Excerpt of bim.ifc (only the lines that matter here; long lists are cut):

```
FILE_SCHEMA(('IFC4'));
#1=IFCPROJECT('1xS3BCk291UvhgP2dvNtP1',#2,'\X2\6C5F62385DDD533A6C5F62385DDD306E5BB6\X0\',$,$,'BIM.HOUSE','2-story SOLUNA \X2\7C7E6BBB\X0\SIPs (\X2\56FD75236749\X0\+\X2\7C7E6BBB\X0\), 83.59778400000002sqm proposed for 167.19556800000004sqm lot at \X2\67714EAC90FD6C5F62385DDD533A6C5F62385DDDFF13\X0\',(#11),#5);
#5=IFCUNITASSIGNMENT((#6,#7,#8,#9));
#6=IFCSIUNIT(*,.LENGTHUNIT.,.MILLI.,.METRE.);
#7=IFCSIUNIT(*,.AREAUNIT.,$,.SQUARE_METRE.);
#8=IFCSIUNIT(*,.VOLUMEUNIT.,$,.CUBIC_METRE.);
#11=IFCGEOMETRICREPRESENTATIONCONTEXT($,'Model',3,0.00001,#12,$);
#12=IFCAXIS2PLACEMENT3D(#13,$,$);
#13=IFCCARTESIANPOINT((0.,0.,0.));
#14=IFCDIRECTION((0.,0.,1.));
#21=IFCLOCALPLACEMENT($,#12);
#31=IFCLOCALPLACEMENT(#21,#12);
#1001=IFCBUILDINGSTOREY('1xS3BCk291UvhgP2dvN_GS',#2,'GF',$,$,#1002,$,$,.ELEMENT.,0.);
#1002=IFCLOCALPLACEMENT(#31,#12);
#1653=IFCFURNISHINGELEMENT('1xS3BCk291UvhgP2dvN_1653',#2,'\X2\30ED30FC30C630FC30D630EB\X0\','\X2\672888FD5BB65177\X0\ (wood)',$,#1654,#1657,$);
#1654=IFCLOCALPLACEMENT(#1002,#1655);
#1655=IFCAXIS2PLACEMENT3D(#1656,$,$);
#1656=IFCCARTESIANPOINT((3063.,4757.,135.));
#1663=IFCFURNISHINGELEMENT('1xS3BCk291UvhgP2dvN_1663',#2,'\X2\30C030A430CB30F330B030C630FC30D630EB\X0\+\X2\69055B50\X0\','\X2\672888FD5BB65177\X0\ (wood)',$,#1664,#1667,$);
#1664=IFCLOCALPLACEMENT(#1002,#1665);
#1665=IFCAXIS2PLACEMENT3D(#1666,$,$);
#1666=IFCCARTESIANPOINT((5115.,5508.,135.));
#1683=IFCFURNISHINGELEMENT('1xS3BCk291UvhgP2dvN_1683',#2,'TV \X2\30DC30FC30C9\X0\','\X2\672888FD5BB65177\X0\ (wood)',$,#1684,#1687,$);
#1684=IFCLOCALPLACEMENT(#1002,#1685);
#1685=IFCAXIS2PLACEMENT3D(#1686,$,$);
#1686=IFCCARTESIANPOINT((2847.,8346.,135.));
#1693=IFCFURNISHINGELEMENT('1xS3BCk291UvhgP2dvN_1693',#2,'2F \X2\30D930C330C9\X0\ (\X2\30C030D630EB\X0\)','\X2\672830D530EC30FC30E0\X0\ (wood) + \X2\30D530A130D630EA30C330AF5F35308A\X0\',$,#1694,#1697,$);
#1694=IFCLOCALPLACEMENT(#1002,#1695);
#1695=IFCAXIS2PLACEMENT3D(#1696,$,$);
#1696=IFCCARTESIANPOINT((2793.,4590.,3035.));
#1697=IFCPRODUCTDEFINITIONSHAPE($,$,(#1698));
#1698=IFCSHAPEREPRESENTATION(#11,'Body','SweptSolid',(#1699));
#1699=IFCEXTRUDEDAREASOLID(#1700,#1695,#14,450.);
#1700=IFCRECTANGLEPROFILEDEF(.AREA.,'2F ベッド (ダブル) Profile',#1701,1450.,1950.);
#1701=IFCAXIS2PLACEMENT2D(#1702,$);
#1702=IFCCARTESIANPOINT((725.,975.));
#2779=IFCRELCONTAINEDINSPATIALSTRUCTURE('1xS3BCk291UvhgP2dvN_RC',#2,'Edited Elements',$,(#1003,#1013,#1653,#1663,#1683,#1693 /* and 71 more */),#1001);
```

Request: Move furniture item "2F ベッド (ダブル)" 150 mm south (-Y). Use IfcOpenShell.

```python
import ifcopenshell
import ifcopenshell.api.geometry
import ifcopenshell.util.placement

model = ifcopenshell.open("bim.ifc")

item = model.by_id(1693)
matrix = ifcopenshell.util.placement.get_local_placement(item.ObjectPlacement)
matrix[1, 3] -= 150.0
ifcopenshell.api.geometry.edit_object_placement(model, product=item, matrix=matrix, is_si=False)

print(ifcopenshell.util.placement.get_local_placement(item.ObjectPlacement).round(3) + 0.0)

model.write("bim_edited.ifc")
```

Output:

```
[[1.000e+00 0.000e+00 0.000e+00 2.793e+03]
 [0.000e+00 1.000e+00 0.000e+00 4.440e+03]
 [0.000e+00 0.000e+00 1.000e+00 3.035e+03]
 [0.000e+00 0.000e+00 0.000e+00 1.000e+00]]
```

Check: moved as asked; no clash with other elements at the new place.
